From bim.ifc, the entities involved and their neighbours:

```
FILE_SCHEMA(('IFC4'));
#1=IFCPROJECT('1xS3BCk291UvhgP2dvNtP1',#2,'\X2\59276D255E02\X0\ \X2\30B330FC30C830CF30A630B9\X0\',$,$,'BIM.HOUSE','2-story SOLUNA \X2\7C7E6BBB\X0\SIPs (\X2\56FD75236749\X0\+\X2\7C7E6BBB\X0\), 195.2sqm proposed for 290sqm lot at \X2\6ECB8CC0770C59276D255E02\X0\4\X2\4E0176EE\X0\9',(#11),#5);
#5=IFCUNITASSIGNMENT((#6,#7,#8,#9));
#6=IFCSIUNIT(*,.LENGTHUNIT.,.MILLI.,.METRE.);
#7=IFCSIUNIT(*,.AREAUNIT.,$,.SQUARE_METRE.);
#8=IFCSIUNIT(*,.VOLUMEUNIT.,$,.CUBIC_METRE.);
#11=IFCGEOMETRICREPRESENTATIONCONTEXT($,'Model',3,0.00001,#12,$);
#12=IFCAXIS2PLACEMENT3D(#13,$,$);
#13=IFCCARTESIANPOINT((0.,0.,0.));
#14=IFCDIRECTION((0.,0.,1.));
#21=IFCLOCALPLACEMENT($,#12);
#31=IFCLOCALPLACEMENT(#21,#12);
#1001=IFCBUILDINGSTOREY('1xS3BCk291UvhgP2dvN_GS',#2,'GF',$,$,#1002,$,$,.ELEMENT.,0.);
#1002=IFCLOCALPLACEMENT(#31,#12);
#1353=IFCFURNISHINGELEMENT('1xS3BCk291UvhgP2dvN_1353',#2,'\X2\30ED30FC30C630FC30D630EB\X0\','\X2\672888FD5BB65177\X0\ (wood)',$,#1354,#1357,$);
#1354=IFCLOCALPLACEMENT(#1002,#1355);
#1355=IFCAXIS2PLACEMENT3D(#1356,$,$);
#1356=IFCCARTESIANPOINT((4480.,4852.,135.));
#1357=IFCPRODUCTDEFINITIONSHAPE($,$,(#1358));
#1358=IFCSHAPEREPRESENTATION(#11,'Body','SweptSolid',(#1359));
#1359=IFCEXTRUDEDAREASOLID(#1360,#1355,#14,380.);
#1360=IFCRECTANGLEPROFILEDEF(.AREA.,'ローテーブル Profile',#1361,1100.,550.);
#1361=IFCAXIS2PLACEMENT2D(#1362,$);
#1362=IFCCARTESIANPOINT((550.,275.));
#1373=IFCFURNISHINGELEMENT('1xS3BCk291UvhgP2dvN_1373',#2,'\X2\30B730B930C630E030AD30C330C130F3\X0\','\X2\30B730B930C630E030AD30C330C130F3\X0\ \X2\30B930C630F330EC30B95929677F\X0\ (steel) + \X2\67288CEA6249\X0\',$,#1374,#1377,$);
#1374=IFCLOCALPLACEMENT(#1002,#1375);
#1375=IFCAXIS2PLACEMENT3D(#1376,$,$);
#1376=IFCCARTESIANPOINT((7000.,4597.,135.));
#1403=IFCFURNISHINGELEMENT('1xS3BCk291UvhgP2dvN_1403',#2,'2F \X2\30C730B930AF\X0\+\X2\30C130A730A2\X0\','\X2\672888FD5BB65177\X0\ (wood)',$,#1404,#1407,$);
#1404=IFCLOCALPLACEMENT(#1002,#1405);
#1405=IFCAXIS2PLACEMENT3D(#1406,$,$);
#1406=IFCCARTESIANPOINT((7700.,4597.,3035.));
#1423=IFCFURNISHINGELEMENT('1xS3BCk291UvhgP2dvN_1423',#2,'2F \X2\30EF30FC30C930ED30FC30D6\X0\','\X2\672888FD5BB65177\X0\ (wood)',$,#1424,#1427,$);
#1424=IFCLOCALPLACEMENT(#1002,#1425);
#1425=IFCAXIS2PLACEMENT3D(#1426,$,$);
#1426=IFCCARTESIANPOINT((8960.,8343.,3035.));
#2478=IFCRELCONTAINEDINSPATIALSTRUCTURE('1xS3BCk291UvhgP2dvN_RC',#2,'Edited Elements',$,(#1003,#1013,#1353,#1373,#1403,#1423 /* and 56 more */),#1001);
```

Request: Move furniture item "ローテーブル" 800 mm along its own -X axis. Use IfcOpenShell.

```python
import ifcopenshell
import ifcopenshell.api.geometry
import ifcopenshell.util.placement
import ifcopenshell.util.unit

model = ifcopenshell.open("bim.ifc")
unit_scale = ifcopenshell.util.unit.calculate_unit_scale(model)

item = model.by_id(1353)
matrix = ifcopenshell.util.placement.get_local_placement(item.ObjectPlacement)
matrix[:3, 3] -= matrix[:3, 0] * 0.8 / unit_scale
ifcopenshell.api.geometry.edit_object_placement(model, product=item, matrix=matrix, is_si=False)

print(ifcopenshell.util.placement.get_local_placement(item.ObjectPlacement).round(3) + 0.0)

model.write("bim_v2.ifc")
```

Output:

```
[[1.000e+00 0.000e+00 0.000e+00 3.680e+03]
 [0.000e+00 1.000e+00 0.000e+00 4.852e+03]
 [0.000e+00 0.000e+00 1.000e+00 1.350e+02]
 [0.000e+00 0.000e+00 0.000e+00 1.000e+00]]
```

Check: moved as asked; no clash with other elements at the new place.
